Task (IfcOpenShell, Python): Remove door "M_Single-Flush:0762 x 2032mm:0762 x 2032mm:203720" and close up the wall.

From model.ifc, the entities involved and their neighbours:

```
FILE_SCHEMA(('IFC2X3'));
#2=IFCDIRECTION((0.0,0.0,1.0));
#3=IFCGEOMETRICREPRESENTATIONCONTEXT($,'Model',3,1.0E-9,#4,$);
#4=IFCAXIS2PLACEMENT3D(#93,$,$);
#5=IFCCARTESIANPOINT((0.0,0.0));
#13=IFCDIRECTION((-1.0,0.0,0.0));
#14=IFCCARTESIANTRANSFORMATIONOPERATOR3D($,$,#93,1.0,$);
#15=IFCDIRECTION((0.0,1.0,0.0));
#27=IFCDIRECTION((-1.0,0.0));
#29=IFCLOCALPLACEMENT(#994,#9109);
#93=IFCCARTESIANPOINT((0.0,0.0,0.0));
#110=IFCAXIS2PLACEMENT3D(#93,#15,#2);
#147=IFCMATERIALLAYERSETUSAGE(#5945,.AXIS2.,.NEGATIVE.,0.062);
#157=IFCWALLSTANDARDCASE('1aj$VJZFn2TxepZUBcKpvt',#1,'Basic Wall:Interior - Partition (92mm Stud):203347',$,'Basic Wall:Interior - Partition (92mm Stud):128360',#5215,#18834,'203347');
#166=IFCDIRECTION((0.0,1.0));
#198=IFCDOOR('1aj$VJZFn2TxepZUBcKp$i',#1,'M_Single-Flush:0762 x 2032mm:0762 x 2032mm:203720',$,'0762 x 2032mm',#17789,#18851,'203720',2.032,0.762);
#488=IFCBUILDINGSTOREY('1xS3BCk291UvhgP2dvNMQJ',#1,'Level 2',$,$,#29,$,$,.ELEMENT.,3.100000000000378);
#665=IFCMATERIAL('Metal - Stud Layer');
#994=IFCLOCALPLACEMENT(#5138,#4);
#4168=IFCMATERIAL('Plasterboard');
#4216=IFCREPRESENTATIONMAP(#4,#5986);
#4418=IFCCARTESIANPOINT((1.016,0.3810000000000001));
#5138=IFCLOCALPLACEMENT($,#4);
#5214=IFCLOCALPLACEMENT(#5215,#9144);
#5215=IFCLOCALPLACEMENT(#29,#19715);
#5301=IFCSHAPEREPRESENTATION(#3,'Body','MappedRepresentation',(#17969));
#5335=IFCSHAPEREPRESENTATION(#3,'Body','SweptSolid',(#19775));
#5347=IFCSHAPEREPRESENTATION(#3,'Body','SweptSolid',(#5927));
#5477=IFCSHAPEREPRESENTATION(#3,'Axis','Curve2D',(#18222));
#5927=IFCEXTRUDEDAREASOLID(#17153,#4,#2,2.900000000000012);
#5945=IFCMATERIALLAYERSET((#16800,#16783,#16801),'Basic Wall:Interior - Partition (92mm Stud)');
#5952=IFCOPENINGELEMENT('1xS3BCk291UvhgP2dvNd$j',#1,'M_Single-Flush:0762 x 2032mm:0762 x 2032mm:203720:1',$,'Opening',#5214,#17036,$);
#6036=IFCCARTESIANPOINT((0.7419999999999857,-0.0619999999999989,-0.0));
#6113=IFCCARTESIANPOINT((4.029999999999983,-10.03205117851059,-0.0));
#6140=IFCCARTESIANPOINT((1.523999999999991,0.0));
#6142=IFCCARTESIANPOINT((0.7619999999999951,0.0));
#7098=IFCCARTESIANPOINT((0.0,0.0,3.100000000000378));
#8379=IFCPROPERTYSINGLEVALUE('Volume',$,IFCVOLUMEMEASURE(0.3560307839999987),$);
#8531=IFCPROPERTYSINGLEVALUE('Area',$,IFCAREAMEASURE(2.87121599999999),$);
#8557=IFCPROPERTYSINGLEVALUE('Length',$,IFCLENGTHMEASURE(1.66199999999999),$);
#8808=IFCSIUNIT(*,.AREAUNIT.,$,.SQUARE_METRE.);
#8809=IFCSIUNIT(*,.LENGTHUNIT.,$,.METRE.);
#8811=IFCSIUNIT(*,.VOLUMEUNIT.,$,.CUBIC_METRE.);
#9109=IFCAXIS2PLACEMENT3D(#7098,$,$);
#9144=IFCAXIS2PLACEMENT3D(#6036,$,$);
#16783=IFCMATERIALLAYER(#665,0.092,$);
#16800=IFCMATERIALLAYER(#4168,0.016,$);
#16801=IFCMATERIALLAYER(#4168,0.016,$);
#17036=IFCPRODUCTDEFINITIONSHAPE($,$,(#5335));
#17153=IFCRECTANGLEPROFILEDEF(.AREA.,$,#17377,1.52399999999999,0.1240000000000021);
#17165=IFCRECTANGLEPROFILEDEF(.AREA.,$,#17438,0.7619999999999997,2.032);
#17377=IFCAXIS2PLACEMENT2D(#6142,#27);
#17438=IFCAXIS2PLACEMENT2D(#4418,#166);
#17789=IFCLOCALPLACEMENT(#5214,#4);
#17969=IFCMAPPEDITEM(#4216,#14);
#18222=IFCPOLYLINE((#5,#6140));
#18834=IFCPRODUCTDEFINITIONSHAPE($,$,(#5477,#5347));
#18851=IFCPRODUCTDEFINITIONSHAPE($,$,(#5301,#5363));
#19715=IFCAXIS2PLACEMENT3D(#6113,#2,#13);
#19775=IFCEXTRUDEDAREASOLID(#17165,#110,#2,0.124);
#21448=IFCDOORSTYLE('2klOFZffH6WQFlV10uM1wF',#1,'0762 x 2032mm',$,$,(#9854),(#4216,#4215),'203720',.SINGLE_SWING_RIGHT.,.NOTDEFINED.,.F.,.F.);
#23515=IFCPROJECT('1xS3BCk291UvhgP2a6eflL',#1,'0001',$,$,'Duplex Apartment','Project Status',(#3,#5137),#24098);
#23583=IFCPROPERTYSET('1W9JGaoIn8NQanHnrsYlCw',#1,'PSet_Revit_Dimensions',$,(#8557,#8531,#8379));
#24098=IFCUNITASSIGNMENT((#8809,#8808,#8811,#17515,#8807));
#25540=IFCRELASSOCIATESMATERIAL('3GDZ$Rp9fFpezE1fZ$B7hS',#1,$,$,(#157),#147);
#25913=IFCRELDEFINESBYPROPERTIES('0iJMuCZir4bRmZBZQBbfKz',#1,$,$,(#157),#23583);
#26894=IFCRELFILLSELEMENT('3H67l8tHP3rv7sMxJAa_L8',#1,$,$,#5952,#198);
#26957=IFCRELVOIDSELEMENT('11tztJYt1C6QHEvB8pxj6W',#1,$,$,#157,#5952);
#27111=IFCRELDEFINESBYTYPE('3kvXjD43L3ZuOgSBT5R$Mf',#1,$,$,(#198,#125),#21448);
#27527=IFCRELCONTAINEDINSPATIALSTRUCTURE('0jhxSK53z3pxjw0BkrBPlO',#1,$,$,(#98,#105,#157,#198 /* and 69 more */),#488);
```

```python
import ifcopenshell
import ifcopenshell.api.feature
import ifcopenshell.api.pset
import ifcopenshell.api.root
import ifcopenshell.geom
import ifcopenshell.util.element
import ifcopenshell.util.shape
import ifcopenshell.util.unit

model = ifcopenshell.open("model.ifc")
area_scale = ifcopenshell.util.unit.calculate_unit_scale(model, "AREAUNIT")
volume_scale = ifcopenshell.util.unit.calculate_unit_scale(model, "VOLUMEUNIT")
settings = ifcopenshell.geom.settings()


def volume(element):
    """Net volume in cubic metres, openings subtracted."""
    shape = ifcopenshell.geom.create_shape(settings, element)
    return ifcopenshell.util.shape.get_volume(shape.geometry)


door = model.by_guid("1aj$VJZFn2TxepZUBcKp$i")
opening = door.FillsVoids[0].RelatingOpeningElement
wall = opening.VoidsElements[0].RelatingBuildingElement
before = volume(wall)

ifcopenshell.api.root.remove_product(model, product=door)
ifcopenshell.api.feature.remove_feature(model, feature=opening)

after = volume(wall)
thickness = 0.124  # wall thickness in metres

# Update the wall's stored quantities.
pset = model.by_id(ifcopenshell.util.element.get_pset(wall, "PSet_Revit_Dimensions", should_inherit=False)["id"])
ifcopenshell.api.pset.edit_pset(model, pset=pset, properties={
    "Area": model.create_entity("IfcAreaMeasure", after / thickness / area_scale),
    "Volume": model.create_entity("IfcVolumeMeasure", after / volume_scale),
})

print(f"wall volume {before:.3f} -> {after:.3f} m3")

model.write("model_v2.ifc")
```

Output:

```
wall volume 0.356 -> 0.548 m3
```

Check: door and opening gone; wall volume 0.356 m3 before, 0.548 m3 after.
